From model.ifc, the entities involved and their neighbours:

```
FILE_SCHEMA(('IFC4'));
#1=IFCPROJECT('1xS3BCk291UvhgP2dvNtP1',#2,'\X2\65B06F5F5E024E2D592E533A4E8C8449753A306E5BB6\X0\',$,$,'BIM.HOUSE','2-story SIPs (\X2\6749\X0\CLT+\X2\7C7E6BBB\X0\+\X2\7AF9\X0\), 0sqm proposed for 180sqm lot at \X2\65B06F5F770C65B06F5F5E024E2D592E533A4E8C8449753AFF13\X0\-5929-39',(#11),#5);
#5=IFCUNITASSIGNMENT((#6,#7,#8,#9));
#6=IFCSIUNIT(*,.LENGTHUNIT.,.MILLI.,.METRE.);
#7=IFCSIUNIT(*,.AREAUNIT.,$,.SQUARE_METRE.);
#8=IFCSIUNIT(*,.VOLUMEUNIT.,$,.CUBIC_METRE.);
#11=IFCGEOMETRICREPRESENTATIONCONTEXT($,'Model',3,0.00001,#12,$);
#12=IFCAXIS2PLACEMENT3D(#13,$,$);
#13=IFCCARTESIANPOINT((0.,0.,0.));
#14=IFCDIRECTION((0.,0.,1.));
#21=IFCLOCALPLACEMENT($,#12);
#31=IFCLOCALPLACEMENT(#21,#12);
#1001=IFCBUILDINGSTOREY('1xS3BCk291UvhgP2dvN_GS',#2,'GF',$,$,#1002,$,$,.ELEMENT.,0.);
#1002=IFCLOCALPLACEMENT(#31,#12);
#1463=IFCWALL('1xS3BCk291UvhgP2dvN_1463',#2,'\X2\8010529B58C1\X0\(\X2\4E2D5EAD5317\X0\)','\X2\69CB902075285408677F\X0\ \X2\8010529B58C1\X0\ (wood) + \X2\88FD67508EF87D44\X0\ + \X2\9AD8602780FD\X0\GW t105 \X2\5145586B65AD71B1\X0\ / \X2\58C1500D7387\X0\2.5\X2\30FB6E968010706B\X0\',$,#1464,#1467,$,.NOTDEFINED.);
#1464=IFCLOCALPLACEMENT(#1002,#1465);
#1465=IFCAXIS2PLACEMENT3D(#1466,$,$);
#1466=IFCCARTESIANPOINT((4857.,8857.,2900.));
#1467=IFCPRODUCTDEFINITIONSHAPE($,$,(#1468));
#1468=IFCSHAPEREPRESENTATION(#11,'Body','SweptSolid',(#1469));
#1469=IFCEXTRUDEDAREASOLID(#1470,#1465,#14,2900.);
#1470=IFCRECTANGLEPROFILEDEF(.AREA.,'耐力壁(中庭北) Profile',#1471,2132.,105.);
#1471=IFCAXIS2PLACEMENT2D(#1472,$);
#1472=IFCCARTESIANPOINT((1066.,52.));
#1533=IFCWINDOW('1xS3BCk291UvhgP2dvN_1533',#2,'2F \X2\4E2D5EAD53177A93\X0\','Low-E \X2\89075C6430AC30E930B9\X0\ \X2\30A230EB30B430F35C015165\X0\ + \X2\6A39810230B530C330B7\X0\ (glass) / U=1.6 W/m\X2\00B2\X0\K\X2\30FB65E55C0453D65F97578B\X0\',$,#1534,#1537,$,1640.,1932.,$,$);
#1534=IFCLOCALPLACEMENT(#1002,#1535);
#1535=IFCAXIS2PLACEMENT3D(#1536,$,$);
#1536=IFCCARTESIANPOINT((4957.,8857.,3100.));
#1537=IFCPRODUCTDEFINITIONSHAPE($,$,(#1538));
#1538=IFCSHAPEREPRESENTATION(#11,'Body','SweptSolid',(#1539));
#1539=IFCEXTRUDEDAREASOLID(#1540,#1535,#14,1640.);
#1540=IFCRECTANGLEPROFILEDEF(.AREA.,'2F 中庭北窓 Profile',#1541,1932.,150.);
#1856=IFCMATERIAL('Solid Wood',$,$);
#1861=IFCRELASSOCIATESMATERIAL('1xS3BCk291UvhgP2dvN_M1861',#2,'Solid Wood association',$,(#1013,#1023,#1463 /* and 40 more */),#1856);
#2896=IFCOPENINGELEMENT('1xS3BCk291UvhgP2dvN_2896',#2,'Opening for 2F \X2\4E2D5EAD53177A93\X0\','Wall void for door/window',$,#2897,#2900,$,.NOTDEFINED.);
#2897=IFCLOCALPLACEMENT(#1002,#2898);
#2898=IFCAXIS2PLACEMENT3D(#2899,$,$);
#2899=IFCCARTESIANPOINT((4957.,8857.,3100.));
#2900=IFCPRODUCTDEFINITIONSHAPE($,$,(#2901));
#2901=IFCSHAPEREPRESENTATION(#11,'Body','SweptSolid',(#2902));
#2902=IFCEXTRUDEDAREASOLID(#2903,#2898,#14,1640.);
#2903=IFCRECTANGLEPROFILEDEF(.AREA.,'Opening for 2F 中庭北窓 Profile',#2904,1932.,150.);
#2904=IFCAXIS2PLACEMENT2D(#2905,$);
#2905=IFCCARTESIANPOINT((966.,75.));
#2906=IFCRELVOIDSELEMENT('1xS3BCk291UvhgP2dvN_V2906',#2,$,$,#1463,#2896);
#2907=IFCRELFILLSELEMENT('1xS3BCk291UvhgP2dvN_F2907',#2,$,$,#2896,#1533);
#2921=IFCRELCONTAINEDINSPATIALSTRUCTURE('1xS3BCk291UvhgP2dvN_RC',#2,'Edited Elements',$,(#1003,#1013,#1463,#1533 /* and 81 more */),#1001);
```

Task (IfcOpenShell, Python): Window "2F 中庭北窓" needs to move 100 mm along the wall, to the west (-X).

```python
import ifcopenshell
import ifcopenshell.api.geometry
import ifcopenshell.util.placement

model = ifcopenshell.open("model.ifc")

window = model.by_guid("1xS3BCk291UvhgP2dvN_1533")
opening = window.FillsVoids[0].RelatingOpeningElement
wall = opening.VoidsElements[0].RelatingBuildingElement

wall_matrix = ifcopenshell.util.placement.get_local_placement(wall.ObjectPlacement)
shift = wall_matrix[:3, 0] * -100.0
before = ifcopenshell.util.placement.get_local_placement(window.ObjectPlacement)[:3, 3].copy()

# The window is not placed relative to its opening, so move both.
for product in (opening, window):
    matrix = ifcopenshell.util.placement.get_local_placement(product.ObjectPlacement)
    matrix[:3, 3] += shift
    ifcopenshell.api.geometry.edit_object_placement(model, product=product, matrix=matrix, is_si=False)

after = ifcopenshell.util.placement.get_local_placement(window.ObjectPlacement)[:3, 3]
print("window moved by", (after - before).round(3) + 0.0)

model.write("model_edited.ifc")
```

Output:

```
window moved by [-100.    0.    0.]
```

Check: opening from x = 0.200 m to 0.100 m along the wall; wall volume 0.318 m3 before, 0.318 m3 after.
